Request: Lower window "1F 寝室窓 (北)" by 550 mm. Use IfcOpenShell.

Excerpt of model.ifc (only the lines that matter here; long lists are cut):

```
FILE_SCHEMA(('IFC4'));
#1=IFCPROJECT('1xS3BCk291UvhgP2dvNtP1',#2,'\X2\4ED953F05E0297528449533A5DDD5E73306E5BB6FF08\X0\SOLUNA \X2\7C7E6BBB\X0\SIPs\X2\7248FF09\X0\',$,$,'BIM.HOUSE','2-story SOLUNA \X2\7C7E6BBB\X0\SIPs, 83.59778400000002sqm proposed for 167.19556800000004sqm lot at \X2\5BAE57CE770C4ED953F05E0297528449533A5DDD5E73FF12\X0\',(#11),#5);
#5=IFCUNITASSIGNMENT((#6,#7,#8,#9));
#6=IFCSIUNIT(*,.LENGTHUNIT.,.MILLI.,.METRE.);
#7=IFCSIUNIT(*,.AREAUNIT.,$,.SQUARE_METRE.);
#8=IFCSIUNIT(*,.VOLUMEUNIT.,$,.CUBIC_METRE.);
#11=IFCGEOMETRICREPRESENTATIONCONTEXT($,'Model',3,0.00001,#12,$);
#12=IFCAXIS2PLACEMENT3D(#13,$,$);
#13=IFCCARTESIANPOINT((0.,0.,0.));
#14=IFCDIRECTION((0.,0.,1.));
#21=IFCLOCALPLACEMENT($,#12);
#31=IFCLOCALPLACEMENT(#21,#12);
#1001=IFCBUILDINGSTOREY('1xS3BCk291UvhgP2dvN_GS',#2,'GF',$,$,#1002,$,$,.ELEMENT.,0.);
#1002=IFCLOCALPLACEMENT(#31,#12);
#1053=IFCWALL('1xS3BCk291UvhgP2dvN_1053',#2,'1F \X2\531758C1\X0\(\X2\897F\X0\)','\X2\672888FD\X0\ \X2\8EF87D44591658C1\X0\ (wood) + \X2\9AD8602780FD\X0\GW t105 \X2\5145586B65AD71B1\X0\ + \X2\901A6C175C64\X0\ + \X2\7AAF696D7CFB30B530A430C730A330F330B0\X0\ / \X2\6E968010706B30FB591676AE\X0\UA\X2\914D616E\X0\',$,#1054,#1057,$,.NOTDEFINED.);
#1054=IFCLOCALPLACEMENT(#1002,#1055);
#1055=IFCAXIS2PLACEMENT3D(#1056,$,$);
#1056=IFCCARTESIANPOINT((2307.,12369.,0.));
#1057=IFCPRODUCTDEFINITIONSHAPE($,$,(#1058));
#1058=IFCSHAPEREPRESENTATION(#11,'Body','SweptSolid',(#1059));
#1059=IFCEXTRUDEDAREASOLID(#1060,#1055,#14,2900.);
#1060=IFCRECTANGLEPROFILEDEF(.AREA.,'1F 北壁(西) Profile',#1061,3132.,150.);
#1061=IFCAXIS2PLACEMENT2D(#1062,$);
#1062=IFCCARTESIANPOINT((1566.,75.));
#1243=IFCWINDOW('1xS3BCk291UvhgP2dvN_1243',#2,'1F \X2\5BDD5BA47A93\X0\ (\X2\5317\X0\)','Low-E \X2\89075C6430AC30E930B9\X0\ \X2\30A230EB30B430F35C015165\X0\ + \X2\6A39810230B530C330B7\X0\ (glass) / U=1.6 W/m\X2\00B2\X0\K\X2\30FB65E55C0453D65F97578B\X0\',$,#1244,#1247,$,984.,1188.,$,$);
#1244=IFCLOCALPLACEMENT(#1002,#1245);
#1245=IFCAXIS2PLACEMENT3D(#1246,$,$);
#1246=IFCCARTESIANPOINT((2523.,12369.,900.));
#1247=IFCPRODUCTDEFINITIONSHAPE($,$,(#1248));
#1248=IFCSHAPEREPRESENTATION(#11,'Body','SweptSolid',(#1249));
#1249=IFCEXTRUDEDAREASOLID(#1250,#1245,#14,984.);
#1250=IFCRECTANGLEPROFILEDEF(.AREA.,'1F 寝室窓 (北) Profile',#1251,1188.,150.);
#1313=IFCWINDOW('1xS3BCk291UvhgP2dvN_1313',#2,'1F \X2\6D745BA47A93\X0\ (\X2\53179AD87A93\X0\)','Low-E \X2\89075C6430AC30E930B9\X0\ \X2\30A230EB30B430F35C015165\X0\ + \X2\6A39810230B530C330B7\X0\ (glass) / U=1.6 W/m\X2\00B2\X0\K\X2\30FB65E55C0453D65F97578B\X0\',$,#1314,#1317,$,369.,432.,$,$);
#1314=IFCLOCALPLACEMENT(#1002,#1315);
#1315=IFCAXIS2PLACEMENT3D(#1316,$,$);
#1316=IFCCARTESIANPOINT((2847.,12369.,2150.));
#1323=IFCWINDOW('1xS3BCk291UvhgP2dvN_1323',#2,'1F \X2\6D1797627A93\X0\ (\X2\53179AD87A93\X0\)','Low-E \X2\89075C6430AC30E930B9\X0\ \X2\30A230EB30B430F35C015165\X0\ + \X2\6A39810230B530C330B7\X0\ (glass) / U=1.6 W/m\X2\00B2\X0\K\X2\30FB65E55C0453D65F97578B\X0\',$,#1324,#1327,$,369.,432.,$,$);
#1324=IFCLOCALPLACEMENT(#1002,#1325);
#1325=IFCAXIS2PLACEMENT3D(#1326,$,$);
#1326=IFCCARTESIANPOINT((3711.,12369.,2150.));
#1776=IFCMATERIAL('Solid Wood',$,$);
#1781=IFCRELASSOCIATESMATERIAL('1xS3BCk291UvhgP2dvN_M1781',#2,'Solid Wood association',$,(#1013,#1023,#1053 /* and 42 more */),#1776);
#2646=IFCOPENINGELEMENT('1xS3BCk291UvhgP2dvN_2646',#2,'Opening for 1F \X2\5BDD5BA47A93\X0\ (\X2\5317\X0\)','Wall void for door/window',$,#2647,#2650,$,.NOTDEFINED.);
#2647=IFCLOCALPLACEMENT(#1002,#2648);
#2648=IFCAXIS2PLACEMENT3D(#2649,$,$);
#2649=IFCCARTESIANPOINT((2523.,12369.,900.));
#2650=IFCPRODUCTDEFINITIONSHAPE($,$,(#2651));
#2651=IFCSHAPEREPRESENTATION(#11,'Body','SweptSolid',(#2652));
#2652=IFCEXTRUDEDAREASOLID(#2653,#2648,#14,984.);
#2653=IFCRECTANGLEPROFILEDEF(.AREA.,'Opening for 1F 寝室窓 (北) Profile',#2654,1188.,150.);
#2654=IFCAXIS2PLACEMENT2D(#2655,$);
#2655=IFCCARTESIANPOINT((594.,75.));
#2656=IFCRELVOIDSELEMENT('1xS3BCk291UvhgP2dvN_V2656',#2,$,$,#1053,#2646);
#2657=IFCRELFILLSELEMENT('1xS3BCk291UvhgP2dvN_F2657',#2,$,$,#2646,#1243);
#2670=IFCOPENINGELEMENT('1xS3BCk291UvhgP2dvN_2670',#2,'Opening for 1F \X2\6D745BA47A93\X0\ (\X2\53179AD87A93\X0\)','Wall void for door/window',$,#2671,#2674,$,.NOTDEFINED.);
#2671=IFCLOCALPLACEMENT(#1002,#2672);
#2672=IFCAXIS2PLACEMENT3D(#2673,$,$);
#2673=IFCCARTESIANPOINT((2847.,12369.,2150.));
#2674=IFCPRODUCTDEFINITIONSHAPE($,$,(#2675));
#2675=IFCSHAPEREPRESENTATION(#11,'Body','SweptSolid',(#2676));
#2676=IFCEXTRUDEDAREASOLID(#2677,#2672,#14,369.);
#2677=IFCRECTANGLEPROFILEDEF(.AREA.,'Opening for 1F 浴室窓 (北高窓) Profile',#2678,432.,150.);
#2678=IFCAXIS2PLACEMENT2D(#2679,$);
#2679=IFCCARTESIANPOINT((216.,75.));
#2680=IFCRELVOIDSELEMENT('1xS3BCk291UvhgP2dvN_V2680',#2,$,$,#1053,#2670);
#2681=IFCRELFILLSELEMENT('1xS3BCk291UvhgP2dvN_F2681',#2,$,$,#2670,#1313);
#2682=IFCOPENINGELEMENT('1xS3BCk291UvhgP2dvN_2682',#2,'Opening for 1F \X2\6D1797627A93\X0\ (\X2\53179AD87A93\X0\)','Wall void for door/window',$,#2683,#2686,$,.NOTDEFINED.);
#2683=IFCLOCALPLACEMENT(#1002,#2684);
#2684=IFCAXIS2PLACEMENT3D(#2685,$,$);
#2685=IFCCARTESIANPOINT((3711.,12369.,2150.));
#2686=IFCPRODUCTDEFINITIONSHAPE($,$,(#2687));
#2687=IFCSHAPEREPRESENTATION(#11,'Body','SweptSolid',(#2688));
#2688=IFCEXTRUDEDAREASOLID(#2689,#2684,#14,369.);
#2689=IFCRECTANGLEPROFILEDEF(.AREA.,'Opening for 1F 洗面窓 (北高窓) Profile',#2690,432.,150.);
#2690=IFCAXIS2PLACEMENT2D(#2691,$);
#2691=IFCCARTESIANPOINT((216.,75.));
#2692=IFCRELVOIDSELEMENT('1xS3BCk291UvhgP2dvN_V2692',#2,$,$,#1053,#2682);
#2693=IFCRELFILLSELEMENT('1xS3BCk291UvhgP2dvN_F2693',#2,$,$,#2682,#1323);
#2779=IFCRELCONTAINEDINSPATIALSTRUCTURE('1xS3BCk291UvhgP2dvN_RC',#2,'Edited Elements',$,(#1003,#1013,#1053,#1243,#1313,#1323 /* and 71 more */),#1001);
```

```python
import numpy as np
import ifcopenshell
import ifcopenshell.api.geometry
import ifcopenshell.util.placement
import ifcopenshell.util.unit

model = ifcopenshell.open("model.ifc")
unit_scale = ifcopenshell.util.unit.calculate_unit_scale(model)

window = model.by_id(1243)
opening = window.FillsVoids[0].RelatingOpeningElement
dz = -0.55 / unit_scale

shift = np.array([0.0, 0.0, dz])
# The window is not placed relative to its opening, so move both.
for product in (opening, window):
    matrix = ifcopenshell.util.placement.get_local_placement(product.ObjectPlacement)
    matrix[:3, 3] += shift
    ifcopenshell.api.geometry.edit_object_placement(model, product=product, matrix=matrix, is_si=False)

print(f"moved by {dz * unit_scale:+.3f} m")

model.write("model_rev.ifc")
```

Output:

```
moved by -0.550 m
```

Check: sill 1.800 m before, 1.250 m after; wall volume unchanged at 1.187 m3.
